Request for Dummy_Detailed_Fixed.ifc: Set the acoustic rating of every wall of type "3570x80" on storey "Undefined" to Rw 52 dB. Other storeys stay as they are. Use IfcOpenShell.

First a look at what the model holds.

```python
import ifcopenshell
import ifcopenshell.util.element

model = ifcopenshell.open("Dummy_Detailed_Fixed.ifc")
print(model.schema)
storey = next(s for s in model.by_type("IfcBuildingStorey") if s.Name == "Undefined")
walls = [e for e in ifcopenshell.util.element.get_decomposition(storey) if e.is_a("IfcWall")]
seen = {}
for e in walls:
    element_type = ifcopenshell.util.element.get_type(e)
    key = (element_type.Name if element_type != e and element_type else None, ifcopenshell.util.element.get_pset(e, "Pset_WallCommon", "AcousticRating"))
    seen[key] = seen.get(key, 0) + 1
for (name, value), count in sorted(seen.items(), key=str):
    print(count, "x", name, "|", value)
```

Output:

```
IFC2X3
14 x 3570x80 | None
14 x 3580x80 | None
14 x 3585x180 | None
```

```python
import ifcopenshell
import ifcopenshell.api.pset
import ifcopenshell.util.element

model = ifcopenshell.open("Dummy_Detailed_Fixed.ifc")

storey = next(s for s in model.by_type("IfcBuildingStorey") if s.Name == "Undefined")
walls = [e for e in ifcopenshell.util.element.get_decomposition(storey) if e.is_a("IfcWall")]

count = 0
for e in walls:
    element_type = ifcopenshell.util.element.get_type(e)
    if element_type in (None, e) or element_type.Name != "3570x80":
        continue
    found = ifcopenshell.util.element.get_pset(e, "Pset_WallCommon", should_inherit=False)
    if found:
        pset = model.by_id(found["id"])
        if len(ifcopenshell.util.element.get_elements_by_pset(pset)) > 1:
            pset = ifcopenshell.api.pset.unshare_pset(model, products=[e], pset=pset)[0]
    else:
        pset = ifcopenshell.api.pset.add_pset(model, product=e, name="Pset_WallCommon")
    ifcopenshell.api.pset.edit_pset(model, pset=pset, properties={"AcousticRating": "Rw 52 dB"})
    count += 1

print(count, "walls updated")

model.write("Dummy_Detailed_Fixed-out.ifc")
```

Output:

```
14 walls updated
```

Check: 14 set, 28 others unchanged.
